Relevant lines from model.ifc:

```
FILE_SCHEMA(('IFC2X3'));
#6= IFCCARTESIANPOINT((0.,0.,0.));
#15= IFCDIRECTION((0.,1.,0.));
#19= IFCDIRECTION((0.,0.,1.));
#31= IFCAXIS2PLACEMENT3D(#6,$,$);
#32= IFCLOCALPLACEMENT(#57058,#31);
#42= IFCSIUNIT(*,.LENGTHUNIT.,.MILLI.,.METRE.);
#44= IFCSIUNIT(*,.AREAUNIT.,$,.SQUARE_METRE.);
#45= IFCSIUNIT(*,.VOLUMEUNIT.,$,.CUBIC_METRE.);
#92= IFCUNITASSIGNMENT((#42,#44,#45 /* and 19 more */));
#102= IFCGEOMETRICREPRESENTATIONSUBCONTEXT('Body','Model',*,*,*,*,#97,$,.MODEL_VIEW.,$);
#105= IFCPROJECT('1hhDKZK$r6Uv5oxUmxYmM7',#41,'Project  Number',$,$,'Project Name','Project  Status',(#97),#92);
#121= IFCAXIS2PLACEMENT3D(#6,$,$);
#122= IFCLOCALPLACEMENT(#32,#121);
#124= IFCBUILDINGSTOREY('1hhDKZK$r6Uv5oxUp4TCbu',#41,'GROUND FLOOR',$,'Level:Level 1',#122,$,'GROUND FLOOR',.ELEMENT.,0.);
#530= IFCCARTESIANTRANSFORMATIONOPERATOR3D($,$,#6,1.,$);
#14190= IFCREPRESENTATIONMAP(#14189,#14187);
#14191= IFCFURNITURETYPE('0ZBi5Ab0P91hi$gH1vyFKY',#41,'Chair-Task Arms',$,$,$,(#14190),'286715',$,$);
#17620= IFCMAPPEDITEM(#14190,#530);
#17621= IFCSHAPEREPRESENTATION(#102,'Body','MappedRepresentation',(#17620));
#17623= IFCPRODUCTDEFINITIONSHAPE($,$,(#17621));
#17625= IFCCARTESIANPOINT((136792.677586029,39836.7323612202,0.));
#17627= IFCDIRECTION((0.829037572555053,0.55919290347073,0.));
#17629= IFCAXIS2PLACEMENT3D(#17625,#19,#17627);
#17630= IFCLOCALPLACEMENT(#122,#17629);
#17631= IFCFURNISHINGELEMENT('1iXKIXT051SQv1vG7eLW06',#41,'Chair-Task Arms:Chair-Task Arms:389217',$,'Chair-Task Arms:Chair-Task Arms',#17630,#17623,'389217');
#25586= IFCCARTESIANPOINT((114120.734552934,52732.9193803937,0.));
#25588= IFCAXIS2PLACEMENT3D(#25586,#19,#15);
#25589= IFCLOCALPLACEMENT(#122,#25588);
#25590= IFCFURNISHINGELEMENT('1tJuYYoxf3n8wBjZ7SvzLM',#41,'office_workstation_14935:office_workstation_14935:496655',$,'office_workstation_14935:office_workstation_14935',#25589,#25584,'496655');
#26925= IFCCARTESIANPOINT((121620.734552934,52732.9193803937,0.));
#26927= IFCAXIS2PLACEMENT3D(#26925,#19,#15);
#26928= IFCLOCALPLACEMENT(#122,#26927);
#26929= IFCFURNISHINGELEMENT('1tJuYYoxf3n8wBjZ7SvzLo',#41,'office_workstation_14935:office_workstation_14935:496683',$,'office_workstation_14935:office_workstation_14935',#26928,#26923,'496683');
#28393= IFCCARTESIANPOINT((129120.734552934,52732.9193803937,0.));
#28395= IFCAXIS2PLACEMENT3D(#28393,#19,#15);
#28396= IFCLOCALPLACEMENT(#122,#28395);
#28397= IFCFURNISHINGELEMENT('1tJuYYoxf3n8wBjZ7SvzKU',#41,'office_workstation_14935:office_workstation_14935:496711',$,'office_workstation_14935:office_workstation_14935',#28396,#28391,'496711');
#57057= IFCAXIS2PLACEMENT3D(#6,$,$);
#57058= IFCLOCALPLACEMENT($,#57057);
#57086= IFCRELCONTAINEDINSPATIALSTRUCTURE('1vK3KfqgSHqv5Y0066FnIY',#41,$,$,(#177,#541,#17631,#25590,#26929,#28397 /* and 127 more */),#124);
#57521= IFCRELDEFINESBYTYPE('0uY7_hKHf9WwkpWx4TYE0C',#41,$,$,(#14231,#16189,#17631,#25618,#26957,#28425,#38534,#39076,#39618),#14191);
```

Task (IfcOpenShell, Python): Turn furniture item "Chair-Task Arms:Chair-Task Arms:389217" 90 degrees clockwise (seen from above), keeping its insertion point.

```python
import ifcopenshell
import ifcopenshell.api.geometry
import ifcopenshell.util.placement

model = ifcopenshell.open("model.ifc")

item = model.by_id(17631)
matrix = ifcopenshell.util.placement.get_local_placement(item.ObjectPlacement)
matrix = matrix @ ifcopenshell.util.placement.rotation(-90, "Z")
ifcopenshell.api.geometry.edit_object_placement(model, product=item, matrix=matrix, is_si=False)

print(ifcopenshell.util.placement.get_local_placement(item.ObjectPlacement).round(3) + 0.0)

model.write("model_rev.ifc")
```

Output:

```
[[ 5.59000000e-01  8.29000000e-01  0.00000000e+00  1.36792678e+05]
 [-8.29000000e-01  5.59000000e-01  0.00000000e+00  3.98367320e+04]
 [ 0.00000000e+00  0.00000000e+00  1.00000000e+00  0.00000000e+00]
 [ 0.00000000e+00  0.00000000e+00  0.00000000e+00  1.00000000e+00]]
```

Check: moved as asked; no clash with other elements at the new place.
